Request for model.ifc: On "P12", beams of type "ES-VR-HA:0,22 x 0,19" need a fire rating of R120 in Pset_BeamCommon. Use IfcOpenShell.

First a look at what the model holds.

```python
import ifcopenshell
import ifcopenshell.util.element

model = ifcopenshell.open("model.ifc")
print(model.schema)
storey = next(s for s in model.by_type("IfcBuildingStorey") if s.Name == "P12")
beams = [e for e in ifcopenshell.util.element.get_decomposition(storey) if e.is_a("IfcBeam")]
seen = {}
for e in beams:
    element_type = ifcopenshell.util.element.get_type(e)
    key = (element_type.Name if element_type != e and element_type else None, ifcopenshell.util.element.get_pset(e, "Pset_BeamCommon", "FireRating"))
    seen[key] = seen.get(key, 0) + 1
for (name, value), count in sorted(seen.items(), key=str):
    print(count, "x", name, "|", value)
```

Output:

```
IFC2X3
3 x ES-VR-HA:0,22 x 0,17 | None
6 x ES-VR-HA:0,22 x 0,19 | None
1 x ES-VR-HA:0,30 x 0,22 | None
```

```python
import ifcopenshell
import ifcopenshell.api.pset
import ifcopenshell.util.element

model = ifcopenshell.open("model.ifc")

storey = next(s for s in model.by_type("IfcBuildingStorey") if s.Name == "P12")
beams = [e for e in ifcopenshell.util.element.get_decomposition(storey) if e.is_a("IfcBeam")]

count = 0
for e in beams:
    element_type = ifcopenshell.util.element.get_type(e)
    if element_type in (None, e) or element_type.Name != "ES-VR-HA:0,22 x 0,19":
        continue
    # add_pset returns the element's existing set when there is one.
    pset = ifcopenshell.api.pset.add_pset(model, product=e, name="Pset_BeamCommon")
    ifcopenshell.api.pset.edit_pset(model, pset=pset, properties={"FireRating": "R120"})
    count += 1

print(count, "beams updated")

model.write("model_rev.ifc")
```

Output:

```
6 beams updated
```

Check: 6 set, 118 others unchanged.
